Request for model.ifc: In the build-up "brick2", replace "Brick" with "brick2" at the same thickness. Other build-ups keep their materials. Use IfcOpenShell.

First a look at what the model holds.

```python
import ifcopenshell
import ifcopenshell.util.element

model = ifcopenshell.open("model.ifc")
print(model.schema)
for layer_set in model.by_type("IfcMaterialLayerSet"):
    if layer_set.LayerSetName == "brick2":
        for layer in layer_set.MaterialLayers:
            print(layer.id(), layer.Material and layer.Material.Name, layer.LayerThickness, sep=" | ")
        print(len(ifcopenshell.util.element.get_elements_by_material(model, layer_set)), "elements and types use it")
print(sorted(m.Name for m in model.by_type("IfcMaterial") if m.Name)[:60])
```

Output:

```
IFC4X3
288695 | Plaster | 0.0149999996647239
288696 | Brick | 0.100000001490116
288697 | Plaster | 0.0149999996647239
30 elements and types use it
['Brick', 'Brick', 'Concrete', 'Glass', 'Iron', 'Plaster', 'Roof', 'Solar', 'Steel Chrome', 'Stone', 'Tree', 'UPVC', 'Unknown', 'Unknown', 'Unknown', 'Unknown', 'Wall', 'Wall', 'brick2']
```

```python
import ifcopenshell
import ifcopenshell.api.material

model = ifcopenshell.open("model.ifc")

layer_set = next(s for s in model.by_type("IfcMaterialLayerSet") if s.LayerSetName == "brick2")
layer = next(l for l in layer_set.MaterialLayers if l.Material and l.Material.Name == "Brick")
material = next(m for m in model.by_type("IfcMaterial") if m.Name == "brick2")

# Point this one layer at the other material; renaming the old one would change it everywhere.
ifcopenshell.api.material.edit_layer(model, layer=layer, attributes={}, material=material)

print([l.Material.Name if l.Material else None for l in layer_set.MaterialLayers])

model.write("model-out.ifc")
```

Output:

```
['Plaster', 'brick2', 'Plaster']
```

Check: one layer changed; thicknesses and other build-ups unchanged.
